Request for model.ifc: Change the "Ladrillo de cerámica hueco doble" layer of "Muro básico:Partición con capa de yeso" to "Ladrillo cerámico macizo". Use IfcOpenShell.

First a look at what the model holds.

```python
import ifcopenshell
import ifcopenshell.util.element

model = ifcopenshell.open("model.ifc")
print(model.schema)
for layer_set in model.by_type("IfcMaterialLayerSet"):
    if layer_set.LayerSetName == "Muro básico:Partición con capa de yeso":
        for layer in layer_set.MaterialLayers:
            print(layer.id(), layer.Material and layer.Material.Name, layer.LayerThickness, sep=" | ")
        print(len(ifcopenshell.util.element.get_elements_by_material(model, layer_set)), "elements and types use it")
print(sorted(m.Name for m in model.by_type("IfcMaterial") if m.Name)[:60])
```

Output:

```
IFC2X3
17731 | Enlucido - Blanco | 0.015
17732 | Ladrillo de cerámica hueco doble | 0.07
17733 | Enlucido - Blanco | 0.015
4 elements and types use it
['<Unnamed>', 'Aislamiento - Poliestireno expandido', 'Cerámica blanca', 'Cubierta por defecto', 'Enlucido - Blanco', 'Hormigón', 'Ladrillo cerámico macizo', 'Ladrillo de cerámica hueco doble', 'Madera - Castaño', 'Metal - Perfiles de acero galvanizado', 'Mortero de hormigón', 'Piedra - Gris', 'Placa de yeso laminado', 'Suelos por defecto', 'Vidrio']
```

```python
import ifcopenshell
import ifcopenshell.api.material

model = ifcopenshell.open("model.ifc")

layer_set = next(s for s in model.by_type("IfcMaterialLayerSet") if s.LayerSetName == "Muro básico:Partición con capa de yeso")
layer = next(l for l in layer_set.MaterialLayers if l.Material and l.Material.Name == "Ladrillo de cerámica hueco doble")
material = next(m for m in model.by_type("IfcMaterial") if m.Name == "Ladrillo cerámico macizo")

# Point this one layer at the other material; renaming the old one would change it everywhere.
ifcopenshell.api.material.edit_layer(model, layer=layer, attributes={}, material=material)

print([l.Material.Name if l.Material else None for l in layer_set.MaterialLayers])

model.write("model_edited.ifc")
```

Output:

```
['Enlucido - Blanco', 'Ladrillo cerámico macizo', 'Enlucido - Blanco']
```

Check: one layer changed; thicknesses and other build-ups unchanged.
